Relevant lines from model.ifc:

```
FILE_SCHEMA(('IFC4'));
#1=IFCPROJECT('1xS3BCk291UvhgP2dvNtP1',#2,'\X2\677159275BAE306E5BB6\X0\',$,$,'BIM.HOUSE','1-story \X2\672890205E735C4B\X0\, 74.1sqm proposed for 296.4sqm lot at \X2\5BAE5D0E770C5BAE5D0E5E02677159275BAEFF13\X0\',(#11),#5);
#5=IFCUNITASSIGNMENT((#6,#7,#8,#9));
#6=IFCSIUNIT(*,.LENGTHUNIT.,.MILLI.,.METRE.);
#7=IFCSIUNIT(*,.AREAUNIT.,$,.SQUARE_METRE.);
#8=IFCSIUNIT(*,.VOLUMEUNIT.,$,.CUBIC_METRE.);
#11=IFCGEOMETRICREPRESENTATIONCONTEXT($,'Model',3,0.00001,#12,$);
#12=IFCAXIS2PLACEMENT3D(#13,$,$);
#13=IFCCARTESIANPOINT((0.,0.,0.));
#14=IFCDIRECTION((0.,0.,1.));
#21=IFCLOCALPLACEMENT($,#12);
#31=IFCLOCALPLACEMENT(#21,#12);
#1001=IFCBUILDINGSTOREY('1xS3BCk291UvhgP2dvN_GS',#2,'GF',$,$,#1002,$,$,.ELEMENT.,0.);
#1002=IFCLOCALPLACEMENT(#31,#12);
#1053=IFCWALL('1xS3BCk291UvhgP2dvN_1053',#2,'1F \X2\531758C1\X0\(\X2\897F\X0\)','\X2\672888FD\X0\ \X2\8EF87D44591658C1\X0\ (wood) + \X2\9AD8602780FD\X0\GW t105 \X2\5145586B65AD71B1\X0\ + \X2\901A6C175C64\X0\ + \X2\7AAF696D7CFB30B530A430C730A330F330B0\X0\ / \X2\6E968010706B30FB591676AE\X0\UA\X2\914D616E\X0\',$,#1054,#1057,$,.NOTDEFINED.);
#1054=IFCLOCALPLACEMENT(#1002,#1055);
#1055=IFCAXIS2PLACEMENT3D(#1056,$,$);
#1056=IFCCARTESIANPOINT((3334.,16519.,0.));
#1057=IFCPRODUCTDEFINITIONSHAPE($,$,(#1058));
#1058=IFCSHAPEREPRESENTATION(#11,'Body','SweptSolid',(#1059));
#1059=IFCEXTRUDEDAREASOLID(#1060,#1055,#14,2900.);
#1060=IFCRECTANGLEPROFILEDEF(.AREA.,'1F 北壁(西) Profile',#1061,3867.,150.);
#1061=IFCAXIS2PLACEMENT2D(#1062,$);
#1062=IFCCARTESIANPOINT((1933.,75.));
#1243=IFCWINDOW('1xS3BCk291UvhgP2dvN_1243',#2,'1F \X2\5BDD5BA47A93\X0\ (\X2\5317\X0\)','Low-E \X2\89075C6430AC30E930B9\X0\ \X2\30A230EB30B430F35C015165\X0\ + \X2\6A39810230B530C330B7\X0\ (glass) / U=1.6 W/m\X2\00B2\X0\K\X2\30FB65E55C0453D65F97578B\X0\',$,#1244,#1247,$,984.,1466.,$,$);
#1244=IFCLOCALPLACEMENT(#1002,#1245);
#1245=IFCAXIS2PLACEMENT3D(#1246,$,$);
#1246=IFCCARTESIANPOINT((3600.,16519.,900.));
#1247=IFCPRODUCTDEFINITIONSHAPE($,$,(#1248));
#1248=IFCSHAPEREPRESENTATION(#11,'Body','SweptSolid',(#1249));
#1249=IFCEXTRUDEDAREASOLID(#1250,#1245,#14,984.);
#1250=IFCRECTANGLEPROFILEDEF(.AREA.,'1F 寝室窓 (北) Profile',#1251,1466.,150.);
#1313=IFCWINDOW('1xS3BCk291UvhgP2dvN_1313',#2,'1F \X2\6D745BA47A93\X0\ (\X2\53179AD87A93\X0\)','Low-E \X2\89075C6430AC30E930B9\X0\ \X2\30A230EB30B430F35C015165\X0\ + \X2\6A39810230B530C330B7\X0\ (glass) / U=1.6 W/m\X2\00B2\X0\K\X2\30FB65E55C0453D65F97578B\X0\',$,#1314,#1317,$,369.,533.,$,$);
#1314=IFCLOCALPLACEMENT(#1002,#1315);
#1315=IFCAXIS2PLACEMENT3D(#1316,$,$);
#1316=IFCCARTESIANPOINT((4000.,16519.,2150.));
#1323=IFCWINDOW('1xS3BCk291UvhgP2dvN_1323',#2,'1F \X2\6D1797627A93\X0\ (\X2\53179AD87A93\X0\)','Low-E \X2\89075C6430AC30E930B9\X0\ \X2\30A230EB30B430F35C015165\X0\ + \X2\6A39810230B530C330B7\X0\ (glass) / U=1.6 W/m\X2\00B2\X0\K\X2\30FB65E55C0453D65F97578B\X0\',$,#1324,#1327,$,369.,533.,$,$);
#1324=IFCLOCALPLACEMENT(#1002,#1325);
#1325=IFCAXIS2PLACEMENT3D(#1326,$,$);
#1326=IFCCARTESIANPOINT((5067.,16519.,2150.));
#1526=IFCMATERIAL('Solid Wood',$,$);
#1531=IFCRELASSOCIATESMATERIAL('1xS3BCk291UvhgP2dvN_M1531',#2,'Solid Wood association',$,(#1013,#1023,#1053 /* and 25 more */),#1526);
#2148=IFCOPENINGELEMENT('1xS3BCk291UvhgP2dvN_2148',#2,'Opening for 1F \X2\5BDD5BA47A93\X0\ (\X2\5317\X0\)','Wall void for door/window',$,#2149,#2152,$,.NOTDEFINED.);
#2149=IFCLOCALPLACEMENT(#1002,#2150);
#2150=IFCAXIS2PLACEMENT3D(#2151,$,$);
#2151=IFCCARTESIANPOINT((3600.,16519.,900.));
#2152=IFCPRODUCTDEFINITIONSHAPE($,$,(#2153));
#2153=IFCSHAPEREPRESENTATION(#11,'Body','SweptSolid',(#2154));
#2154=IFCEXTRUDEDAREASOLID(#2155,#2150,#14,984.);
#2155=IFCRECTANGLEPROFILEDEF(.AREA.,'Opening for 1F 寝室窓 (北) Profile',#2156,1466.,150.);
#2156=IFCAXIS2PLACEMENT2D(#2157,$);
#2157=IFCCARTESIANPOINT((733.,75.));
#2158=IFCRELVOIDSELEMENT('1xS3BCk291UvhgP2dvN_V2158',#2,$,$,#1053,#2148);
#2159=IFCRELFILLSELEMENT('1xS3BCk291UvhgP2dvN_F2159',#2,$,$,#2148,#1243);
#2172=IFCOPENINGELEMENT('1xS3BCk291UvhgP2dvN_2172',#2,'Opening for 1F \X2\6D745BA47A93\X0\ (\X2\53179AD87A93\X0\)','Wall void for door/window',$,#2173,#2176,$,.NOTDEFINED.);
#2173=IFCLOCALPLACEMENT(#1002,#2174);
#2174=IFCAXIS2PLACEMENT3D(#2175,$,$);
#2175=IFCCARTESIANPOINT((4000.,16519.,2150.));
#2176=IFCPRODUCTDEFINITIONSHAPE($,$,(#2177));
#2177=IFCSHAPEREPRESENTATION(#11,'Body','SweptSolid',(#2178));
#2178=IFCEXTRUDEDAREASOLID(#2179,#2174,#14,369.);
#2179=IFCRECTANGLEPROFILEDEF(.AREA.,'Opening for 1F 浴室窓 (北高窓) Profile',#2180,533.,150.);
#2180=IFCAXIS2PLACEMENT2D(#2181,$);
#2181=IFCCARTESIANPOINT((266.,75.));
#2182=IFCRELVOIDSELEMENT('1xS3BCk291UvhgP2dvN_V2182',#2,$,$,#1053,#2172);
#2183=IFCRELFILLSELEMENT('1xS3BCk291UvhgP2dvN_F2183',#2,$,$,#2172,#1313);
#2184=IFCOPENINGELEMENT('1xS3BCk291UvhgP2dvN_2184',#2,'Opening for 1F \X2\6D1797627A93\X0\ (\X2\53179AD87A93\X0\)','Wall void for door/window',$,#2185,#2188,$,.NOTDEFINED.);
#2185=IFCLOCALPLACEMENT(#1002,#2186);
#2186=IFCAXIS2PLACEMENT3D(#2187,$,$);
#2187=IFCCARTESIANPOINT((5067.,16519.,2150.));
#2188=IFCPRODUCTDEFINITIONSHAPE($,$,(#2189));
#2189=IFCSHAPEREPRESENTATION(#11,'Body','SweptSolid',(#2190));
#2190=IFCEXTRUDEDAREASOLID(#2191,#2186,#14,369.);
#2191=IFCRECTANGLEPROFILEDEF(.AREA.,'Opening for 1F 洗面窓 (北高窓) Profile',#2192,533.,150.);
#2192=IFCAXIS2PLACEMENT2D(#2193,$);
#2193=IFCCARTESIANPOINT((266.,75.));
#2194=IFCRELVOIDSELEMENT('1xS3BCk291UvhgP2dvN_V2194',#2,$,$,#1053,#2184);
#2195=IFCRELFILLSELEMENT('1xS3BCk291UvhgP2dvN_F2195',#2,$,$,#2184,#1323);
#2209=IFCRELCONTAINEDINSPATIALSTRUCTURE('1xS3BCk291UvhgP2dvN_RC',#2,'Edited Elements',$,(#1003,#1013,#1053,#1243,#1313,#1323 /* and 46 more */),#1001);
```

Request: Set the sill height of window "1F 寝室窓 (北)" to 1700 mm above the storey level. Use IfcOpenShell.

```python
import numpy as np
import ifcopenshell
import ifcopenshell.api.geometry
import ifcopenshell.geom
import ifcopenshell.util.element
import ifcopenshell.util.placement
import ifcopenshell.util.shape
import ifcopenshell.util.unit

model = ifcopenshell.open("model.ifc")
unit_scale = ifcopenshell.util.unit.calculate_unit_scale(model)

window = model.by_guid("1xS3BCk291UvhgP2dvN_1243")
opening = window.FillsVoids[0].RelatingOpeningElement
storey = ifcopenshell.util.element.get_container(window, ifc_class="IfcBuildingStorey")
level = ifcopenshell.util.placement.get_local_placement(storey.ObjectPlacement)[2, 3]

# The opening's origin need not be at the sill, so measure its lowest point.
shape = ifcopenshell.geom.create_shape(ifcopenshell.geom.settings(), opening)
bottom = ifcopenshell.util.shape.get_shape_bottom_elevation(shape, shape.geometry) / unit_scale
dz = level + 1700.0 - bottom

shift = np.array([0.0, 0.0, dz])
# The window is not placed relative to its opening, so move both.
for product in (opening, window):
    matrix = ifcopenshell.util.placement.get_local_placement(product.ObjectPlacement)
    matrix[:3, 3] += shift
    ifcopenshell.api.geometry.edit_object_placement(model, product=product, matrix=matrix, is_si=False)

print(f"moved by {dz * unit_scale:+.3f} m")

model.write("model_edited.ifc")
```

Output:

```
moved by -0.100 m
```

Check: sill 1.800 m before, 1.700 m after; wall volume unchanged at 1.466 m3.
